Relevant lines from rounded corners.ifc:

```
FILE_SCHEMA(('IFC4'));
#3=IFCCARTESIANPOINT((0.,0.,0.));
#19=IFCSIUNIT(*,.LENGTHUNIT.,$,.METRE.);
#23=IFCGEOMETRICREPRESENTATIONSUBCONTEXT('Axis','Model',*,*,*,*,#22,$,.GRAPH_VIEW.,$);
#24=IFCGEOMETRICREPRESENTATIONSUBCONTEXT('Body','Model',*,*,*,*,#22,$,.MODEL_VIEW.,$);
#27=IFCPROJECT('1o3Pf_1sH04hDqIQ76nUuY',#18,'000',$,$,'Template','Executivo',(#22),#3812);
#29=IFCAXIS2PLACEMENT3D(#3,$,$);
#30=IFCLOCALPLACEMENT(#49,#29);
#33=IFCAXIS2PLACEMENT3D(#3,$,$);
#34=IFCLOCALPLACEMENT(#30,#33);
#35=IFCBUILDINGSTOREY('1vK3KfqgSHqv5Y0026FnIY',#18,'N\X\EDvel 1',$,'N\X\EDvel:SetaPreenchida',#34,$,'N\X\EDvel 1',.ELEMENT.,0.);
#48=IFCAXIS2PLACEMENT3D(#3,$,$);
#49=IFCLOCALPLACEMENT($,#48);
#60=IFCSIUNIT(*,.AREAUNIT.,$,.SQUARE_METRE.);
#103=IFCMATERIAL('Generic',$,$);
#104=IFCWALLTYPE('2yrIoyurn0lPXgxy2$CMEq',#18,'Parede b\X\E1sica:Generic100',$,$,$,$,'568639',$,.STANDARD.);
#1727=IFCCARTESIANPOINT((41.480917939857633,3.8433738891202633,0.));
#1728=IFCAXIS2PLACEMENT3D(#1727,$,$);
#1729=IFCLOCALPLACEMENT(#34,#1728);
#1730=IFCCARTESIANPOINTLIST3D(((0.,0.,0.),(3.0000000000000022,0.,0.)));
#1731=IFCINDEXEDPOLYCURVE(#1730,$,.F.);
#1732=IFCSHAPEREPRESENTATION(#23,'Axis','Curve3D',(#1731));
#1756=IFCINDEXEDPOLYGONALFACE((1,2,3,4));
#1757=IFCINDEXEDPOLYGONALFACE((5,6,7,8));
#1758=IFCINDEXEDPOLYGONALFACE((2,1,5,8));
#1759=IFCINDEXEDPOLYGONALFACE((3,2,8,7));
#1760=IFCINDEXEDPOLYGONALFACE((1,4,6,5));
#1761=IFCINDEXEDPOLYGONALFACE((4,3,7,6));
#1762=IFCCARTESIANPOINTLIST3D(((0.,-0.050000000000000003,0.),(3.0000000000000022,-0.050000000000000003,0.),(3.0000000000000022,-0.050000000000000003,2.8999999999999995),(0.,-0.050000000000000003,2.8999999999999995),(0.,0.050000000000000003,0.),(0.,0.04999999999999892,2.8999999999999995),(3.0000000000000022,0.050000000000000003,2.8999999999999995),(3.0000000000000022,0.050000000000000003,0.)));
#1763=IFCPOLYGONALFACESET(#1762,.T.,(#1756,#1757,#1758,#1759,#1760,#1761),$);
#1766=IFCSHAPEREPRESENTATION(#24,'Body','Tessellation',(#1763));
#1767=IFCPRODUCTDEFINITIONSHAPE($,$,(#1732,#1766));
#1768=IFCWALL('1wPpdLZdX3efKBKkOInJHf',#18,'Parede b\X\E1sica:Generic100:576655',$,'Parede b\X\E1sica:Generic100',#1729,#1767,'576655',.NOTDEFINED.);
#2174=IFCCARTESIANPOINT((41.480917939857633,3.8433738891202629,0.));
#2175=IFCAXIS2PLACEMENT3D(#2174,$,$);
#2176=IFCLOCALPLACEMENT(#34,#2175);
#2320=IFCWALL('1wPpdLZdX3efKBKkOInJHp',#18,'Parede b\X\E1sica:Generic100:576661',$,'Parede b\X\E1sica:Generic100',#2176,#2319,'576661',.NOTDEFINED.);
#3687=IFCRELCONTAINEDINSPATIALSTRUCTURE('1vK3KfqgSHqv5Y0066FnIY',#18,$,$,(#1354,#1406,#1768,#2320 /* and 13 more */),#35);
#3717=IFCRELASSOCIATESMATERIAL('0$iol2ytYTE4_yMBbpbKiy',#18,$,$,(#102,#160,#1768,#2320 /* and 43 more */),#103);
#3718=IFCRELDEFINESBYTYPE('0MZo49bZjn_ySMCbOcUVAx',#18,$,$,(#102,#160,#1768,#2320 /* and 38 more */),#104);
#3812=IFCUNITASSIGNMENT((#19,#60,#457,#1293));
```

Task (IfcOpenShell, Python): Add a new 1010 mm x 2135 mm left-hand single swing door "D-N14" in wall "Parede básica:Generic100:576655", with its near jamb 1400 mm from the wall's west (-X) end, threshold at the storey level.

```python
import numpy as np
import ifcopenshell
import ifcopenshell.api.feature
import ifcopenshell.api.geometry
import ifcopenshell.api.root
import ifcopenshell.api.spatial
import ifcopenshell.geom
import ifcopenshell.util.element
import ifcopenshell.util.placement
import ifcopenshell.util.representation
import ifcopenshell.util.shape
import ifcopenshell.util.unit

model = ifcopenshell.open("rounded corners.ifc")
unit_scale = ifcopenshell.util.unit.calculate_unit_scale(model)
settings = ifcopenshell.geom.settings()


def volume(element):
    """Net volume in cubic metres, openings subtracted."""
    shape = ifcopenshell.geom.create_shape(settings, element)
    return ifcopenshell.util.shape.get_volume(shape.geometry)


wall = model.by_guid("1wPpdLZdX3efKBKkOInJHf")
storey = ifcopenshell.util.element.get_container(wall, ifc_class="IfcBuildingStorey")
context = ifcopenshell.util.representation.get_context(model, "Model", "Body", "MODEL_VIEW")
before = volume(wall)

width, height, from_end, sill = 1.01, 2.135, 1.4, 0.0  # metres

# The wall runs along its own X axis, and the end named is its -X end.
wall_shape = ifcopenshell.geom.create_shape(settings, wall)
x, y, z = ifcopenshell.util.shape.get_vertices(wall_shape.geometry).T
start = x.min() + from_end
face, thickness = float(y.min()), float(y.max() - y.min())
wall_matrix = ifcopenshell.util.placement.get_local_placement(wall.ObjectPlacement)
level = ifcopenshell.util.placement.get_local_placement(storey.ObjectPlacement)[2, 3]


def in_wall(x, y):
    """Placement at x, y metres in the wall's axes, at sill height."""
    matrix = wall_matrix.copy()
    matrix[:, 3] = wall_matrix @ np.array([x / unit_scale, y / unit_scale, 0.0, 1.0])
    matrix[2, 3] = level + sill / unit_scale
    return matrix


# Opening: a box that overshoots both wall faces by 50 mm.
opening = ifcopenshell.api.root.create_entity(model, ifc_class="IfcOpeningElement", predefined_type="OPENING")
box = ifcopenshell.api.geometry.add_wall_representation(
    model, context=context, length=width, height=height, thickness=thickness + 0.1
)
ifcopenshell.api.geometry.assign_representation(model, product=opening, representation=box)
ifcopenshell.api.geometry.edit_object_placement(model, product=opening, matrix=in_wall(start, face - 0.05), is_si=False)
ifcopenshell.api.feature.add_feature(model, feature=opening, element=wall)

door = ifcopenshell.api.root.create_entity(model, ifc_class="IfcDoor", name="D-N14", predefined_type="DOOR")
door.OverallWidth, door.OverallHeight = width / unit_scale, height / unit_scale
door.OperationType = "SINGLE_SWING_LEFT"
body = ifcopenshell.api.geometry.add_door_representation(
    model,
    context=context,
    overall_width=door.OverallWidth,
    overall_height=door.OverallHeight,
    operation_type="SINGLE_SWING_LEFT",
    lining_properties={"LiningDepth": thickness / unit_scale, "ThresholdDepth": thickness / unit_scale},
)
ifcopenshell.api.geometry.assign_representation(model, product=door, representation=body)
ifcopenshell.api.spatial.assign_container(model, products=[door], relating_structure=storey)
ifcopenshell.api.feature.add_filling(model, opening=opening, element=door)

# The lining spans the wall, so the door starts at the wall face.
ifcopenshell.api.geometry.edit_object_placement(model, product=door, matrix=in_wall(start, face), is_si=False)

after = volume(wall)

print(f"wall volume {before:.3f} -> {after:.3f} m3")

model.write("rounded corners_rev.ifc")
```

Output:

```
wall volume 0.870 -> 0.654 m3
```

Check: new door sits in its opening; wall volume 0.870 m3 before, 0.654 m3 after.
